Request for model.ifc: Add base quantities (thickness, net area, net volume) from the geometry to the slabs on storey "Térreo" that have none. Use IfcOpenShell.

First a look at what the model holds.

```python
import ifcopenshell
import ifcopenshell.util.element
import ifcopenshell.util.unit

model = ifcopenshell.open("model.ifc")
print(model.schema)
for unit_type in ("LENGTHUNIT", "AREAUNIT", "VOLUMEUNIT"):
    print(unit_type, ifcopenshell.util.unit.calculate_unit_scale(model, unit_type))
storey = next(s for s in model.by_type("IfcBuildingStorey") if s.Name == "Térreo")
slabs = [e for e in ifcopenshell.util.element.get_decomposition(storey) if e.is_a("IfcSlab")]
for e in sorted(slabs, key=lambda e: e.id()):
    print(e.id(), e.is_a(), e.Name, list(ifcopenshell.util.element.get_psets(e, qtos_only=True)), sep=" | ")
```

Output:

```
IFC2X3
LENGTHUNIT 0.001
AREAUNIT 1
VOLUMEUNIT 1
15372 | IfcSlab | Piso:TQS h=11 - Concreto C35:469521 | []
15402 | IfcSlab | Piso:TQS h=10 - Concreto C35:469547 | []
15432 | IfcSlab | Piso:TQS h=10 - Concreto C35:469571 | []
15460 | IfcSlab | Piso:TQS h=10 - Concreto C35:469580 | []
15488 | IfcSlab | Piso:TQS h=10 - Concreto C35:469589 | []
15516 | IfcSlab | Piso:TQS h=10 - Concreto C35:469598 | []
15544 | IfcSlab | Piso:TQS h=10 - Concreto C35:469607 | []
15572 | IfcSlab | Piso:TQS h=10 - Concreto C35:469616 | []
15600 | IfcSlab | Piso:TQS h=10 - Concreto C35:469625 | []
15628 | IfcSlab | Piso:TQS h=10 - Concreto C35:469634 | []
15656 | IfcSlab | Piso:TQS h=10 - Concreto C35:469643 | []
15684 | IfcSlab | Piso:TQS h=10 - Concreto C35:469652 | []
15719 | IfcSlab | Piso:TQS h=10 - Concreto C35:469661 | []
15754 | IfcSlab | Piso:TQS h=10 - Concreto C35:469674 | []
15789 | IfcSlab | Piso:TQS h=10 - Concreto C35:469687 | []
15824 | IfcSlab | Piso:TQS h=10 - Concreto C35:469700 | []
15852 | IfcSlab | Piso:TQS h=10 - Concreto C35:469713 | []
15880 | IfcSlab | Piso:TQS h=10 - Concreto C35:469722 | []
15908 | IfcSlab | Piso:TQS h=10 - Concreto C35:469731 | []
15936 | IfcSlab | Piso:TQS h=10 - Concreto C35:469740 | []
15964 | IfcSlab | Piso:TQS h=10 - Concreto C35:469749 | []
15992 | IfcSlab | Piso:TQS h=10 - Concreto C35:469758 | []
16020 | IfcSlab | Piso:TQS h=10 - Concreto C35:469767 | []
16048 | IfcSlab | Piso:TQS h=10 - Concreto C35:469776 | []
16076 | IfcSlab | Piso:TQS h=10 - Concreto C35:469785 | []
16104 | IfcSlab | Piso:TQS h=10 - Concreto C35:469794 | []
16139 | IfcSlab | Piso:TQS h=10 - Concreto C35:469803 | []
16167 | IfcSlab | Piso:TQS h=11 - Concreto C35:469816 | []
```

```python
import ifcopenshell
import ifcopenshell.api.pset
import ifcopenshell.geom
import ifcopenshell.util.element
import ifcopenshell.util.shape
import ifcopenshell.util.unit

model = ifcopenshell.open("model.ifc")
unit_scale = ifcopenshell.util.unit.calculate_unit_scale(model)
area_scale = ifcopenshell.util.unit.calculate_unit_scale(model, "AREAUNIT")
volume_scale = ifcopenshell.util.unit.calculate_unit_scale(model, "VOLUMEUNIT")
settings = ifcopenshell.geom.settings()

storey = next(s for s in model.by_type("IfcBuildingStorey") if s.Name == "Térreo")
slabs = [e for e in ifcopenshell.util.element.get_decomposition(storey) if e.is_a("IfcSlab")]

for e in sorted(slabs, key=lambda e: e.id()):
    if ifcopenshell.util.element.get_psets(e, qtos_only=True, should_inherit=False):
        continue
    # Geometry comes back in metres, in the element's own axes.
    shape = ifcopenshell.geom.create_shape(settings, e)
    values = {
        "Width": ifcopenshell.util.shape.get_z(shape.geometry) / unit_scale,
        "NetArea": ifcopenshell.util.shape.get_footprint_area(shape.geometry) / area_scale,
        "NetVolume": ifcopenshell.util.shape.get_volume(shape.geometry) / volume_scale,
    }
    qto = ifcopenshell.api.pset.add_qto(model, product=e, name="BaseQuantities")
    ifcopenshell.api.pset.edit_qto(model, qto=qto, properties=values)
    print(e.id(), {k: round(v, 3) for k, v in values.items()})

model.write("model_updated.ifc")
```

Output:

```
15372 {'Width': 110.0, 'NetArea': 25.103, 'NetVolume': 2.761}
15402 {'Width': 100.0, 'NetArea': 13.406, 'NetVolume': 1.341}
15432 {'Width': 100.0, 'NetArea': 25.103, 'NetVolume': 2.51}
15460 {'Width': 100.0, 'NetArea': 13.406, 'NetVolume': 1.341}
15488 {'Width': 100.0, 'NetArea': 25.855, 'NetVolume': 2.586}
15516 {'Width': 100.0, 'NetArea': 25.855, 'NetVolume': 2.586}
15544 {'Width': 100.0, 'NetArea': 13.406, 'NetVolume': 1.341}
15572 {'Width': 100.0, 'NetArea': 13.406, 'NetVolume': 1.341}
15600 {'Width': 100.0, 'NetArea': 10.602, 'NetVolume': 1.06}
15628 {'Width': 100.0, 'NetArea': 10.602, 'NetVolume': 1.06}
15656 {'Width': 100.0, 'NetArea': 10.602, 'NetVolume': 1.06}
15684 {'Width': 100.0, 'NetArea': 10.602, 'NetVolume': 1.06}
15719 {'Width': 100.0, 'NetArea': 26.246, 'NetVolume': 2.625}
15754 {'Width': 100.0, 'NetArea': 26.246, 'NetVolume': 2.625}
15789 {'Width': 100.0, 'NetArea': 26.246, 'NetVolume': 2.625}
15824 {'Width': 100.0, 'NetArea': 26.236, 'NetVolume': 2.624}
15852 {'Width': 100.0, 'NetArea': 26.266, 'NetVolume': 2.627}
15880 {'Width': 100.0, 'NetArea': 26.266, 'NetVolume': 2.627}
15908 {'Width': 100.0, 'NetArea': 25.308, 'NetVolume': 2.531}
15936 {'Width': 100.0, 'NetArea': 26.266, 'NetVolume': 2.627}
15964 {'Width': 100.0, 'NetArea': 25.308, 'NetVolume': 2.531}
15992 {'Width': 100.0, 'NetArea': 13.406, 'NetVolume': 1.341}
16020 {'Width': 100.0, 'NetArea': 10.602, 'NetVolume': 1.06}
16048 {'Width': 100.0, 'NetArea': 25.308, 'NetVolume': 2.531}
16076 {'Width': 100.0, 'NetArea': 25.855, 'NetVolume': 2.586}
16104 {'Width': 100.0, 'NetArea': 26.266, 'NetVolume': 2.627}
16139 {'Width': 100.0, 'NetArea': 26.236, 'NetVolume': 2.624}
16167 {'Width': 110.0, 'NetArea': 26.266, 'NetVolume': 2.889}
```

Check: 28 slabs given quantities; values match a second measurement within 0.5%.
